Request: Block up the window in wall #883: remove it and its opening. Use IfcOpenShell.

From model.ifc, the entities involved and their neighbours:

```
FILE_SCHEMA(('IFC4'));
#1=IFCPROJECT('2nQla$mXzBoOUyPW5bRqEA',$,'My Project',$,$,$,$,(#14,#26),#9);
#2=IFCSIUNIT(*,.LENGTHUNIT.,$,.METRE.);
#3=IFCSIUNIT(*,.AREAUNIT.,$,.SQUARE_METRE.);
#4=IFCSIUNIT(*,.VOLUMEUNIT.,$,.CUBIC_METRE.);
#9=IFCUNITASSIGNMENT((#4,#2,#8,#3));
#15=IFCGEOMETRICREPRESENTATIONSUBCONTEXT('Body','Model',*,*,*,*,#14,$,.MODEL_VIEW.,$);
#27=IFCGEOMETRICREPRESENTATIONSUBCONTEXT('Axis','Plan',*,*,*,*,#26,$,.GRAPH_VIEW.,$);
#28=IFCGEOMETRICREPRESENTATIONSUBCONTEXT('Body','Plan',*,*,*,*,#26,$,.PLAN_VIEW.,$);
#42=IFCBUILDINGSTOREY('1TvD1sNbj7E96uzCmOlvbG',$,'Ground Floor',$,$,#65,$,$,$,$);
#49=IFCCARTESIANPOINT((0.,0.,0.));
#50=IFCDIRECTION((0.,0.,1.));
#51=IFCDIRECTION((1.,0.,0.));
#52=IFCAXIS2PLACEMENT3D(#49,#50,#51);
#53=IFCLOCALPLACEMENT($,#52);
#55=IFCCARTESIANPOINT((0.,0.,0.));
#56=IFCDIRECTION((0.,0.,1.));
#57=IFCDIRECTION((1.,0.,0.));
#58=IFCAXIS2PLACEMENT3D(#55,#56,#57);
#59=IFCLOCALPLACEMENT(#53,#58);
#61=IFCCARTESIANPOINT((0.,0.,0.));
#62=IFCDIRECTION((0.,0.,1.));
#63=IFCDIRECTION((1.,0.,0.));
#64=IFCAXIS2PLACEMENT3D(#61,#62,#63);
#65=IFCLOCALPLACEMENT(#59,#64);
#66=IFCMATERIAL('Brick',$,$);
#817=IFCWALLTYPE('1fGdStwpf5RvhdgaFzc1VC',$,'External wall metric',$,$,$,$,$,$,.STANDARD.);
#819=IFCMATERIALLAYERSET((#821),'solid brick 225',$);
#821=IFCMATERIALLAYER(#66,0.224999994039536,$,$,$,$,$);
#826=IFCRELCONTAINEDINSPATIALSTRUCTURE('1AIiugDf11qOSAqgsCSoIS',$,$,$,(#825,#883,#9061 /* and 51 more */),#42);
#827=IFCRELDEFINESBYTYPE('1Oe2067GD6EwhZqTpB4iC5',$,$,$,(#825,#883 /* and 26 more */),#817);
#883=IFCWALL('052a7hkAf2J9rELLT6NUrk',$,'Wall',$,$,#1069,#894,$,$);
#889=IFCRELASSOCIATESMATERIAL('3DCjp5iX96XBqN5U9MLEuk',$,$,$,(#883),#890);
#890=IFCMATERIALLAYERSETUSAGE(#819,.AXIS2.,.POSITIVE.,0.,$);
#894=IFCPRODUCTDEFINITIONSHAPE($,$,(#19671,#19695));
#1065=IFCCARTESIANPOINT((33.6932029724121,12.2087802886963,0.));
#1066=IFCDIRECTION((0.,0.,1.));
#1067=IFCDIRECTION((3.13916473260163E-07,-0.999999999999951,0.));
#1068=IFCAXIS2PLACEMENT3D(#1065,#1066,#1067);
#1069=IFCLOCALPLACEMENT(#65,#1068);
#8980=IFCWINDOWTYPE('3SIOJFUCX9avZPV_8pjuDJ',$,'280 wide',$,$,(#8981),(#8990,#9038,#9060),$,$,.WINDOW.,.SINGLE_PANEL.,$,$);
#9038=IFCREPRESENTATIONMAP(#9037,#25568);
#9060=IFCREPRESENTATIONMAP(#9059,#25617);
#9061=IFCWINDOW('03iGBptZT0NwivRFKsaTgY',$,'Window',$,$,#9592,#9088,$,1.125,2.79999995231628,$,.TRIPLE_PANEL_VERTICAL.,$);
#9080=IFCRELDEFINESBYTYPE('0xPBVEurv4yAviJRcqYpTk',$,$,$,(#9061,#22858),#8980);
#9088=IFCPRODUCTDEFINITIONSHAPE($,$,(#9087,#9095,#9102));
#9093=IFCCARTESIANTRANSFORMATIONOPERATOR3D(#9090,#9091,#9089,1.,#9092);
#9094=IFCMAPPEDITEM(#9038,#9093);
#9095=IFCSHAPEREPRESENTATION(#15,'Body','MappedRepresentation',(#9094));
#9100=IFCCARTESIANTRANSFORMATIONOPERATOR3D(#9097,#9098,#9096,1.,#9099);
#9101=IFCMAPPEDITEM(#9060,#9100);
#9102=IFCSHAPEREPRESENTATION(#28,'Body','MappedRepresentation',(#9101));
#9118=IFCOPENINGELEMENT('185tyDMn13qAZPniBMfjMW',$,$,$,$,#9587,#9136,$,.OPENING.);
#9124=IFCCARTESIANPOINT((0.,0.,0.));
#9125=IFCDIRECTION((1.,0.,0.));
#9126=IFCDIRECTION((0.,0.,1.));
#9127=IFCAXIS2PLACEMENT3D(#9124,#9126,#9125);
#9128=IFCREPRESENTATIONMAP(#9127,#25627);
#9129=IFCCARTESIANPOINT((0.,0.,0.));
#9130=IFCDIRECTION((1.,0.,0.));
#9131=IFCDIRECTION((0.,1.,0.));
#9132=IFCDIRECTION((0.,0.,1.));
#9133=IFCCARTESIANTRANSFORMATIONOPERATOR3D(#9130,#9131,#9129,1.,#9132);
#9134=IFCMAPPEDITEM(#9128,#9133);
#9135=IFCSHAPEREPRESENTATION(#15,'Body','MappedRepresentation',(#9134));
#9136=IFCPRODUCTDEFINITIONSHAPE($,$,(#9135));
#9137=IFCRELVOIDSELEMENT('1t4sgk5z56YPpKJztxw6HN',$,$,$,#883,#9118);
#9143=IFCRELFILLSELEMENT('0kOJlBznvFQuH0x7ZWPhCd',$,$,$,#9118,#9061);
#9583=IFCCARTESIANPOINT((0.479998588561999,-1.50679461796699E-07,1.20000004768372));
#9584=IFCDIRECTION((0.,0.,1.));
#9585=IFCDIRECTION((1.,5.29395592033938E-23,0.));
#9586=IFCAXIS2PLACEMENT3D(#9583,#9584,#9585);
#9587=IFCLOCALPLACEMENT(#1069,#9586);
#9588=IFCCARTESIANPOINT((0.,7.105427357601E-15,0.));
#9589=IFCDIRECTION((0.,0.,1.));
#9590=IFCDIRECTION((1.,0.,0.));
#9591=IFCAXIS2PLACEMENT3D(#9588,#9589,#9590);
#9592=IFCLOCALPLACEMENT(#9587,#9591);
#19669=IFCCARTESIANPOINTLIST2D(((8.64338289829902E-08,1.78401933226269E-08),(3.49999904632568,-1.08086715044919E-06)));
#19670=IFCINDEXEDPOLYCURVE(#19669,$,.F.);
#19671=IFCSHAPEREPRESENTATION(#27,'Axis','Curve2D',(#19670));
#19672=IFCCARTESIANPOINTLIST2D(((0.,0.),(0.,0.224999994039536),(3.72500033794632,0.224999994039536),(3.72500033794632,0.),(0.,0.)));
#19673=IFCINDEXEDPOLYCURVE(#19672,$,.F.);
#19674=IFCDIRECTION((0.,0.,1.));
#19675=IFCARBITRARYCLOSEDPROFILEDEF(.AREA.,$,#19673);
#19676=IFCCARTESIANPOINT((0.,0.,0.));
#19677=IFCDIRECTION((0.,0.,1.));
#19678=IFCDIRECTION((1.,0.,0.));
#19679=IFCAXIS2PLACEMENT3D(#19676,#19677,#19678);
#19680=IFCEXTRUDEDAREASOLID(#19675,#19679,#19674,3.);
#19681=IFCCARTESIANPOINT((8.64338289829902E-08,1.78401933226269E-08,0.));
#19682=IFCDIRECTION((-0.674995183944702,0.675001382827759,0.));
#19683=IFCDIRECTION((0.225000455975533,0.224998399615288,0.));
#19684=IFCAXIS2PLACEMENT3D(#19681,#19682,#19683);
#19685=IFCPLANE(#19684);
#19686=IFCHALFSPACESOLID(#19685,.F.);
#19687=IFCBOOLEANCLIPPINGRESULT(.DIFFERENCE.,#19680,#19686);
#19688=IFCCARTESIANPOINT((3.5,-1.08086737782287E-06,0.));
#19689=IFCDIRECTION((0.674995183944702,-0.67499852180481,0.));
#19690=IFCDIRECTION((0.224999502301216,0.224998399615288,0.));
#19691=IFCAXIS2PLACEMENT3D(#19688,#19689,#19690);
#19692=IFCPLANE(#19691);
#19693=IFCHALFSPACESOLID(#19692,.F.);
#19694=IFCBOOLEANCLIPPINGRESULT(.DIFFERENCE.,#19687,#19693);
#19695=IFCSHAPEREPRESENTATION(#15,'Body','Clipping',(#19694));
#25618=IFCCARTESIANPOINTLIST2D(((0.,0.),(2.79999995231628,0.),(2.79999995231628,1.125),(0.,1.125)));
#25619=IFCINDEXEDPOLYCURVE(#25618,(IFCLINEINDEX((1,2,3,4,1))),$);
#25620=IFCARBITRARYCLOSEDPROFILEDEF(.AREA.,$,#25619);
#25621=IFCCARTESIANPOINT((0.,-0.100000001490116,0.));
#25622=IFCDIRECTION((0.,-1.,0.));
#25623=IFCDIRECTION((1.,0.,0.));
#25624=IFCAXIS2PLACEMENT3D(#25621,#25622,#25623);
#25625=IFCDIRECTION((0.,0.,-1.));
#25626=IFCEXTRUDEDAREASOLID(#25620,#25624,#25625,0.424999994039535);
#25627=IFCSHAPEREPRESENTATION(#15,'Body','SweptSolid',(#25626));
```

```python
import ifcopenshell
import ifcopenshell.api.feature
import ifcopenshell.api.root
import ifcopenshell.geom
import ifcopenshell.util.shape

model = ifcopenshell.open("model.ifc")
settings = ifcopenshell.geom.settings()


def volume(element):
    """Net volume in cubic metres, openings subtracted."""
    shape = ifcopenshell.geom.create_shape(settings, element)
    return ifcopenshell.util.shape.get_volume(shape.geometry)


window = model.by_guid("03iGBptZT0NwivRFKsaTgY")
opening = window.FillsVoids[0].RelatingOpeningElement
wall = opening.VoidsElements[0].RelatingBuildingElement
before = volume(wall)

ifcopenshell.api.root.remove_product(model, product=window)
ifcopenshell.api.feature.remove_feature(model, feature=opening)

after = volume(wall)

print(f"wall volume {before:.3f} -> {after:.3f} m3")

model.write("model_v2.ifc")
```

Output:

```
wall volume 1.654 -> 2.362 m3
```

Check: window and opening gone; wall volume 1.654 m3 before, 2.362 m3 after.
